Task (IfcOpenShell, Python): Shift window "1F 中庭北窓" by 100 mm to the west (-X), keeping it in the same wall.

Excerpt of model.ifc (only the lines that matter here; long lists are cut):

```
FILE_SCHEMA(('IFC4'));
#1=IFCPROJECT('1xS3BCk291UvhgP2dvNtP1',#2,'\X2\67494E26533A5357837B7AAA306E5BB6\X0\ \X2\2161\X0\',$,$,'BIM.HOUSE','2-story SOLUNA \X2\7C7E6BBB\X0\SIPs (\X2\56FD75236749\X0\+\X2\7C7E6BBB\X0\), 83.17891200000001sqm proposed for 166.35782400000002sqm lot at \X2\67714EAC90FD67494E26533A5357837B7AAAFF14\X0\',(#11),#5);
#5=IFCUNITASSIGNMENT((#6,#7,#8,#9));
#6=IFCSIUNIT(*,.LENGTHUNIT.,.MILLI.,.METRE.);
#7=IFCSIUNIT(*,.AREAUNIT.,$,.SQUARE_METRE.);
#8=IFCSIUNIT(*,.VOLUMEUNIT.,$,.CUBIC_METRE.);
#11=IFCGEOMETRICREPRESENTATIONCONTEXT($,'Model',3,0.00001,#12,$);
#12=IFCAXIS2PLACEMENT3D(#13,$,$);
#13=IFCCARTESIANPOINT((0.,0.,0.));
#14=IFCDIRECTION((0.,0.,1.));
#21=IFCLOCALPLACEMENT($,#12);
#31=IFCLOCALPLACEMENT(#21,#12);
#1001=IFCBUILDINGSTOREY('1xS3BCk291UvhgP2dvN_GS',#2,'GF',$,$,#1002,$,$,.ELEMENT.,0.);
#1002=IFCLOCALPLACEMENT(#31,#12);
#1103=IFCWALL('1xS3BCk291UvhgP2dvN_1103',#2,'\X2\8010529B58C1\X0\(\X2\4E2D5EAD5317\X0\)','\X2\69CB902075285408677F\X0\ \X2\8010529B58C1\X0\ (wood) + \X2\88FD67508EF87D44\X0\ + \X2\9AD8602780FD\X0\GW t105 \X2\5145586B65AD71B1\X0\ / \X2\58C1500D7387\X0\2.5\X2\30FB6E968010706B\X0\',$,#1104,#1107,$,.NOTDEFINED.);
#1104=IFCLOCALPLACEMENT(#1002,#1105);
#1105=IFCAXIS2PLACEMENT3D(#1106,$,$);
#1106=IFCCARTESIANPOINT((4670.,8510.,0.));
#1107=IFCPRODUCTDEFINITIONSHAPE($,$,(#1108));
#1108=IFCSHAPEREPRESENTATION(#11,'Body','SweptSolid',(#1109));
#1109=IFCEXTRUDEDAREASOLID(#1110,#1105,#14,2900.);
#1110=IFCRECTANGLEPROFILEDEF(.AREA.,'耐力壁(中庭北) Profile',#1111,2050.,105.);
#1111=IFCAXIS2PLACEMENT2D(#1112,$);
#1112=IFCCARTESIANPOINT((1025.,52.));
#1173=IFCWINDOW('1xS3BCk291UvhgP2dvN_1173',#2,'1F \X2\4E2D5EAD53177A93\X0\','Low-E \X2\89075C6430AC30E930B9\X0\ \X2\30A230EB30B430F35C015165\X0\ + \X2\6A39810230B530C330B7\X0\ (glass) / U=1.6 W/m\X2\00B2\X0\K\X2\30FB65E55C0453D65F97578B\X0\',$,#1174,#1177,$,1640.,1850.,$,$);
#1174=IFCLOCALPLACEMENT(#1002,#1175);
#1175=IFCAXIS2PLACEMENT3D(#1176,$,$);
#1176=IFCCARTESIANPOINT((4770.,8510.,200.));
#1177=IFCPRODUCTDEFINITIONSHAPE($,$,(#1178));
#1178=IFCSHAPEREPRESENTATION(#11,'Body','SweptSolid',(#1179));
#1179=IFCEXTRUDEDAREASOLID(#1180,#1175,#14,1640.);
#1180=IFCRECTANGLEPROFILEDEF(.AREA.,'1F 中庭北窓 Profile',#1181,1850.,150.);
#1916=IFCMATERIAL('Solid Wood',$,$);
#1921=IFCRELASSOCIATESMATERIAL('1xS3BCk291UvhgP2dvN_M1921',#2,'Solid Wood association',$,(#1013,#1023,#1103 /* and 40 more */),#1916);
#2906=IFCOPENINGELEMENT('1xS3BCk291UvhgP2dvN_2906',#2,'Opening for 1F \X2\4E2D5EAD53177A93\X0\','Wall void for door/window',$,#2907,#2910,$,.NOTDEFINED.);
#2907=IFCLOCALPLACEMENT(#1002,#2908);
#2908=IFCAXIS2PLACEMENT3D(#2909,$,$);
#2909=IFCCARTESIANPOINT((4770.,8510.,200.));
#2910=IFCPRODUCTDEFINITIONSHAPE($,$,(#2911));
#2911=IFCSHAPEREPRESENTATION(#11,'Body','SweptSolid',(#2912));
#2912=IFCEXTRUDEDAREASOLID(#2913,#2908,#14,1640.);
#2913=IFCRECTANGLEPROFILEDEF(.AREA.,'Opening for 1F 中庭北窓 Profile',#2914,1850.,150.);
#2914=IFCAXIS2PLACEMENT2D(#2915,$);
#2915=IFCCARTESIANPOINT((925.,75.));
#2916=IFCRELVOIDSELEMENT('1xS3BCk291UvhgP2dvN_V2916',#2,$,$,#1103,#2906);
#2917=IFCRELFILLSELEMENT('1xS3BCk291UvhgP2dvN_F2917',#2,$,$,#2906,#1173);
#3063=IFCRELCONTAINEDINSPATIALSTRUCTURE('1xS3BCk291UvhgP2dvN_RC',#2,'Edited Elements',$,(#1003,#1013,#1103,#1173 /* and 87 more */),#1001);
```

```python
import ifcopenshell
import ifcopenshell.api.geometry
import ifcopenshell.util.placement
import ifcopenshell.util.unit

model = ifcopenshell.open("model.ifc")
unit_scale = ifcopenshell.util.unit.calculate_unit_scale(model)

window = model.by_guid("1xS3BCk291UvhgP2dvN_1173")
opening = window.FillsVoids[0].RelatingOpeningElement
wall = opening.VoidsElements[0].RelatingBuildingElement

wall_matrix = ifcopenshell.util.placement.get_local_placement(wall.ObjectPlacement)
shift = wall_matrix[:3, 0] * -0.1 / unit_scale
before = ifcopenshell.util.placement.get_local_placement(window.ObjectPlacement)[:3, 3].copy()

# The window is not placed relative to its opening, so move both.
for product in (opening, window):
    matrix = ifcopenshell.util.placement.get_local_placement(product.ObjectPlacement)
    matrix[:3, 3] += shift
    ifcopenshell.api.geometry.edit_object_placement(model, product=product, matrix=matrix, is_si=False)

after = ifcopenshell.util.placement.get_local_placement(window.ObjectPlacement)[:3, 3]
print("window moved by", (after - before).round(3) + 0.0)

model.write("model_rev.ifc")
```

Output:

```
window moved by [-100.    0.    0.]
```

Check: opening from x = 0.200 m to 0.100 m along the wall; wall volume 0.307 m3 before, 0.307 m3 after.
